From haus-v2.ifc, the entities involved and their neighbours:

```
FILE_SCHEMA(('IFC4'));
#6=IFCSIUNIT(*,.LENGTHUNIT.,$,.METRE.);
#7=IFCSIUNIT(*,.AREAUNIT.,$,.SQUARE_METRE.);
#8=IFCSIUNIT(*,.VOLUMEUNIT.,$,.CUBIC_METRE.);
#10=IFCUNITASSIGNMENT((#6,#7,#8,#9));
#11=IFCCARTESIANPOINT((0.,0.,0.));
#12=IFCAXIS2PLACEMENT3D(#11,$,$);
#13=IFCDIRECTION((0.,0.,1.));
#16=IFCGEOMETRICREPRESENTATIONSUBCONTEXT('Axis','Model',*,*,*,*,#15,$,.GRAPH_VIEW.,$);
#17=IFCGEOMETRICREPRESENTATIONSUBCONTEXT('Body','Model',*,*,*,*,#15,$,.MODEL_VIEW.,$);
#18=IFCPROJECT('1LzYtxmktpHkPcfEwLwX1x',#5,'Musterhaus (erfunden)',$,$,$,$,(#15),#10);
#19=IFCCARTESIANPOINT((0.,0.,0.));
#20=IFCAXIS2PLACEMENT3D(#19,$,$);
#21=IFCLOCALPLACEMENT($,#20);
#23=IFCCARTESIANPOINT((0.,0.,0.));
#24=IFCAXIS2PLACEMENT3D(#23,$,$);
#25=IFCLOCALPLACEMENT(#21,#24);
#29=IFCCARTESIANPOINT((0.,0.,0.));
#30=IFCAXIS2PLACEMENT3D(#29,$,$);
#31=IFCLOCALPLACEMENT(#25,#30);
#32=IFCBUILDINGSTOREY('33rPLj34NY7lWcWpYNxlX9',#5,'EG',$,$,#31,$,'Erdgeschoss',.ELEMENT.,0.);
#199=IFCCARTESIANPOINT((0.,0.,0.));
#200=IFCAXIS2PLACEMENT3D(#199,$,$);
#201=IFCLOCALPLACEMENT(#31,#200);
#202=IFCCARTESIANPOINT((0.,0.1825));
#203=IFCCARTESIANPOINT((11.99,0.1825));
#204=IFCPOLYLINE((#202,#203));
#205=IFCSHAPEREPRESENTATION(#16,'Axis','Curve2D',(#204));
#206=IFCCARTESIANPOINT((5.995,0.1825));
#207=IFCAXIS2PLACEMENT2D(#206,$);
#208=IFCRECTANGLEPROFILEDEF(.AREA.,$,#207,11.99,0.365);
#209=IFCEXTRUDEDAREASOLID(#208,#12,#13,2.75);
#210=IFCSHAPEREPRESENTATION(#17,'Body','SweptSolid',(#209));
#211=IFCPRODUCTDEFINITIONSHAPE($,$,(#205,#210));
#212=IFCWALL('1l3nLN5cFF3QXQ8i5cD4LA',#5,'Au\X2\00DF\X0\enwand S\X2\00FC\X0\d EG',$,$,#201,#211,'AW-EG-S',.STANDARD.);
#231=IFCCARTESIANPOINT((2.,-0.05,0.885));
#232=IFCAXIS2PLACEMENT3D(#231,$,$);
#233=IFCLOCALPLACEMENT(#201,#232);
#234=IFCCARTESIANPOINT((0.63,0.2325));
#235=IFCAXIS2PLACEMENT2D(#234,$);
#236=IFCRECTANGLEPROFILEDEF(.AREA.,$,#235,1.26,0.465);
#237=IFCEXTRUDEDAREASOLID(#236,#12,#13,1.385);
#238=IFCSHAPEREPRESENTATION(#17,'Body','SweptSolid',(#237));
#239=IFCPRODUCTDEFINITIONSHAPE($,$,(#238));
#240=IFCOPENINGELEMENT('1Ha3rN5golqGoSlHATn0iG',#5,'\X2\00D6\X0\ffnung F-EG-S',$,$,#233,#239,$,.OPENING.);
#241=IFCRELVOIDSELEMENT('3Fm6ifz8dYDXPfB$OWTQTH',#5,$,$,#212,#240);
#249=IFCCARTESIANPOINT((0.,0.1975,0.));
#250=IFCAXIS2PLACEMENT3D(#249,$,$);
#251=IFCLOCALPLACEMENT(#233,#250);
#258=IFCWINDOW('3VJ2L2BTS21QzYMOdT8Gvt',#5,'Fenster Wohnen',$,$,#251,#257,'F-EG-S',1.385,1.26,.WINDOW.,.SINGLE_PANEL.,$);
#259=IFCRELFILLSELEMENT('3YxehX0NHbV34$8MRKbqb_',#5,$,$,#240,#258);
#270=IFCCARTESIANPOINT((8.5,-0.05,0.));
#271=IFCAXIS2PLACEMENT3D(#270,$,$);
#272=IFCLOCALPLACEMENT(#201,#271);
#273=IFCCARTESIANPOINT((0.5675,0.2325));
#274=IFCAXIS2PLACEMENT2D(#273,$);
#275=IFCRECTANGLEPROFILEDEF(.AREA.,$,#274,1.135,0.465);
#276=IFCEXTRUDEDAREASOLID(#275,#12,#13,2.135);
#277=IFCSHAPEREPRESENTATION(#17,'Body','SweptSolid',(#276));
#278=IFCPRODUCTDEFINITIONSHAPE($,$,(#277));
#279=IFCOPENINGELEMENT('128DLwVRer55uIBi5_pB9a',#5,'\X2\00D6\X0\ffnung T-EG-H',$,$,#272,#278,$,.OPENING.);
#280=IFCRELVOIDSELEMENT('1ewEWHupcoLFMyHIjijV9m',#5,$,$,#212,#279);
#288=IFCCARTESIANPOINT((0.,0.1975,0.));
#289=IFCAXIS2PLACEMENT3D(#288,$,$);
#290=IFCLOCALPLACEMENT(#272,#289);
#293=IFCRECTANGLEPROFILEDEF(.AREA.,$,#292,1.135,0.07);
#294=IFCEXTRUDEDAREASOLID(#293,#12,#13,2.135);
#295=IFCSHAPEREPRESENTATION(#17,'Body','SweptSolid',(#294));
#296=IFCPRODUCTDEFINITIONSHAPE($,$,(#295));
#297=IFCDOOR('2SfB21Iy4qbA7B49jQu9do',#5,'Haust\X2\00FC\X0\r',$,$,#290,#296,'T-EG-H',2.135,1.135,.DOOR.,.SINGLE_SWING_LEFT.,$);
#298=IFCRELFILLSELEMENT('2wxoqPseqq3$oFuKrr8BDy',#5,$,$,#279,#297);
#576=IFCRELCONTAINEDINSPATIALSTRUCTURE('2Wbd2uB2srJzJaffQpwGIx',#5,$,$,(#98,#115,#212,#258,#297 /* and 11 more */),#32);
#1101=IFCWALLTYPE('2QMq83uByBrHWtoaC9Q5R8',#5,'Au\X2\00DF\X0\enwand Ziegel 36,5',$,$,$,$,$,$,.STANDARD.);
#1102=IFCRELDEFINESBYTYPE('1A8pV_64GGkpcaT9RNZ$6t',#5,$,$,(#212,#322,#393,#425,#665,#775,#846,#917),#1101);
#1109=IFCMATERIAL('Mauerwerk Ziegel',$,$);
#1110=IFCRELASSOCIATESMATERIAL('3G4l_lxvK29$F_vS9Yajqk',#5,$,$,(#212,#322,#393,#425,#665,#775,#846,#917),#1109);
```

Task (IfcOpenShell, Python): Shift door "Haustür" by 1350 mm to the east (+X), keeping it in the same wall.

```python
import ifcopenshell
import ifcopenshell.api.geometry
import ifcopenshell.util.placement
import ifcopenshell.util.unit

model = ifcopenshell.open("haus-v2.ifc")
unit_scale = ifcopenshell.util.unit.calculate_unit_scale(model)

door = model.by_guid("2SfB21Iy4qbA7B49jQu9do")
opening = door.FillsVoids[0].RelatingOpeningElement
wall = opening.VoidsElements[0].RelatingBuildingElement

wall_matrix = ifcopenshell.util.placement.get_local_placement(wall.ObjectPlacement)
shift = wall_matrix[:3, 0] * 1.35 / unit_scale
before = ifcopenshell.util.placement.get_local_placement(door.ObjectPlacement)[:3, 3].copy()

# The door is placed relative to its opening, so it follows when the opening moves.
matrix = ifcopenshell.util.placement.get_local_placement(opening.ObjectPlacement)
matrix[:3, 3] += shift
ifcopenshell.api.geometry.edit_object_placement(
    model, product=opening, matrix=matrix, is_si=False, should_transform_children=True
)

after = ifcopenshell.util.placement.get_local_placement(door.ObjectPlacement)[:3, 3]
print("door moved by", (after - before).round(3) + 0.0)

model.write("haus-v2_v2.ifc")
```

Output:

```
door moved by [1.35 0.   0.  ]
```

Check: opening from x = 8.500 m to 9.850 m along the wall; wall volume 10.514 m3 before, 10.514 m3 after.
